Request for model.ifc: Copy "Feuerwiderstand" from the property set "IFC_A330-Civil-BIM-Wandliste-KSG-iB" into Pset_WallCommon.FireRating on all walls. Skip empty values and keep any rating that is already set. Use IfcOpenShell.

First a look at what the model holds.

```python
import ifcopenshell
import ifcopenshell.util.element

model = ifcopenshell.open("model.ifc")
print(model.schema)
walls = model.by_type("IfcWall")
print(len(walls), "walls")
for e in walls[:8]:
    source = ifcopenshell.util.element.get_pset(e, "IFC_A330-Civil-BIM-Wandliste-KSG-iB", "Feuerwiderstand")
    target = ifcopenshell.util.element.get_pset(e, "Pset_WallCommon", "FireRating")
    print(e.id(), repr(source), repr(target), sep=" | ")
```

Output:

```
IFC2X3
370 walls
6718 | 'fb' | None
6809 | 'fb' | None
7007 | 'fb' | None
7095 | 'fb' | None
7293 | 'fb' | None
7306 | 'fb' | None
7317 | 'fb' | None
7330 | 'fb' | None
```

```python
import ifcopenshell
import ifcopenshell.api.pset
import ifcopenshell.util.element

model = ifcopenshell.open("model.ifc")

count = 0
for e in model.by_type("IfcWall"):
    value = ifcopenshell.util.element.get_pset(e, "IFC_A330-Civil-BIM-Wandliste-KSG-iB", "Feuerwiderstand")
    current = ifcopenshell.util.element.get_pset(e, "Pset_WallCommon", "FireRating")
    if not value or not value.strip() or current:
        continue
    found = ifcopenshell.util.element.get_pset(e, "Pset_WallCommon", should_inherit=False)
    if found:
        pset = model.by_id(found["id"])
        if len(ifcopenshell.util.element.get_elements_by_pset(pset)) > 1:
            pset = ifcopenshell.api.pset.unshare_pset(model, products=[e], pset=pset)[0]
    else:
        pset = ifcopenshell.api.pset.add_pset(model, product=e, name="Pset_WallCommon")
    ifcopenshell.api.pset.edit_pset(model, pset=pset, properties={"FireRating": value})
    count += 1

print(count, "walls updated")

model.write("model-out.ifc")
```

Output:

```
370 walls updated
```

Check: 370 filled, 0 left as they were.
